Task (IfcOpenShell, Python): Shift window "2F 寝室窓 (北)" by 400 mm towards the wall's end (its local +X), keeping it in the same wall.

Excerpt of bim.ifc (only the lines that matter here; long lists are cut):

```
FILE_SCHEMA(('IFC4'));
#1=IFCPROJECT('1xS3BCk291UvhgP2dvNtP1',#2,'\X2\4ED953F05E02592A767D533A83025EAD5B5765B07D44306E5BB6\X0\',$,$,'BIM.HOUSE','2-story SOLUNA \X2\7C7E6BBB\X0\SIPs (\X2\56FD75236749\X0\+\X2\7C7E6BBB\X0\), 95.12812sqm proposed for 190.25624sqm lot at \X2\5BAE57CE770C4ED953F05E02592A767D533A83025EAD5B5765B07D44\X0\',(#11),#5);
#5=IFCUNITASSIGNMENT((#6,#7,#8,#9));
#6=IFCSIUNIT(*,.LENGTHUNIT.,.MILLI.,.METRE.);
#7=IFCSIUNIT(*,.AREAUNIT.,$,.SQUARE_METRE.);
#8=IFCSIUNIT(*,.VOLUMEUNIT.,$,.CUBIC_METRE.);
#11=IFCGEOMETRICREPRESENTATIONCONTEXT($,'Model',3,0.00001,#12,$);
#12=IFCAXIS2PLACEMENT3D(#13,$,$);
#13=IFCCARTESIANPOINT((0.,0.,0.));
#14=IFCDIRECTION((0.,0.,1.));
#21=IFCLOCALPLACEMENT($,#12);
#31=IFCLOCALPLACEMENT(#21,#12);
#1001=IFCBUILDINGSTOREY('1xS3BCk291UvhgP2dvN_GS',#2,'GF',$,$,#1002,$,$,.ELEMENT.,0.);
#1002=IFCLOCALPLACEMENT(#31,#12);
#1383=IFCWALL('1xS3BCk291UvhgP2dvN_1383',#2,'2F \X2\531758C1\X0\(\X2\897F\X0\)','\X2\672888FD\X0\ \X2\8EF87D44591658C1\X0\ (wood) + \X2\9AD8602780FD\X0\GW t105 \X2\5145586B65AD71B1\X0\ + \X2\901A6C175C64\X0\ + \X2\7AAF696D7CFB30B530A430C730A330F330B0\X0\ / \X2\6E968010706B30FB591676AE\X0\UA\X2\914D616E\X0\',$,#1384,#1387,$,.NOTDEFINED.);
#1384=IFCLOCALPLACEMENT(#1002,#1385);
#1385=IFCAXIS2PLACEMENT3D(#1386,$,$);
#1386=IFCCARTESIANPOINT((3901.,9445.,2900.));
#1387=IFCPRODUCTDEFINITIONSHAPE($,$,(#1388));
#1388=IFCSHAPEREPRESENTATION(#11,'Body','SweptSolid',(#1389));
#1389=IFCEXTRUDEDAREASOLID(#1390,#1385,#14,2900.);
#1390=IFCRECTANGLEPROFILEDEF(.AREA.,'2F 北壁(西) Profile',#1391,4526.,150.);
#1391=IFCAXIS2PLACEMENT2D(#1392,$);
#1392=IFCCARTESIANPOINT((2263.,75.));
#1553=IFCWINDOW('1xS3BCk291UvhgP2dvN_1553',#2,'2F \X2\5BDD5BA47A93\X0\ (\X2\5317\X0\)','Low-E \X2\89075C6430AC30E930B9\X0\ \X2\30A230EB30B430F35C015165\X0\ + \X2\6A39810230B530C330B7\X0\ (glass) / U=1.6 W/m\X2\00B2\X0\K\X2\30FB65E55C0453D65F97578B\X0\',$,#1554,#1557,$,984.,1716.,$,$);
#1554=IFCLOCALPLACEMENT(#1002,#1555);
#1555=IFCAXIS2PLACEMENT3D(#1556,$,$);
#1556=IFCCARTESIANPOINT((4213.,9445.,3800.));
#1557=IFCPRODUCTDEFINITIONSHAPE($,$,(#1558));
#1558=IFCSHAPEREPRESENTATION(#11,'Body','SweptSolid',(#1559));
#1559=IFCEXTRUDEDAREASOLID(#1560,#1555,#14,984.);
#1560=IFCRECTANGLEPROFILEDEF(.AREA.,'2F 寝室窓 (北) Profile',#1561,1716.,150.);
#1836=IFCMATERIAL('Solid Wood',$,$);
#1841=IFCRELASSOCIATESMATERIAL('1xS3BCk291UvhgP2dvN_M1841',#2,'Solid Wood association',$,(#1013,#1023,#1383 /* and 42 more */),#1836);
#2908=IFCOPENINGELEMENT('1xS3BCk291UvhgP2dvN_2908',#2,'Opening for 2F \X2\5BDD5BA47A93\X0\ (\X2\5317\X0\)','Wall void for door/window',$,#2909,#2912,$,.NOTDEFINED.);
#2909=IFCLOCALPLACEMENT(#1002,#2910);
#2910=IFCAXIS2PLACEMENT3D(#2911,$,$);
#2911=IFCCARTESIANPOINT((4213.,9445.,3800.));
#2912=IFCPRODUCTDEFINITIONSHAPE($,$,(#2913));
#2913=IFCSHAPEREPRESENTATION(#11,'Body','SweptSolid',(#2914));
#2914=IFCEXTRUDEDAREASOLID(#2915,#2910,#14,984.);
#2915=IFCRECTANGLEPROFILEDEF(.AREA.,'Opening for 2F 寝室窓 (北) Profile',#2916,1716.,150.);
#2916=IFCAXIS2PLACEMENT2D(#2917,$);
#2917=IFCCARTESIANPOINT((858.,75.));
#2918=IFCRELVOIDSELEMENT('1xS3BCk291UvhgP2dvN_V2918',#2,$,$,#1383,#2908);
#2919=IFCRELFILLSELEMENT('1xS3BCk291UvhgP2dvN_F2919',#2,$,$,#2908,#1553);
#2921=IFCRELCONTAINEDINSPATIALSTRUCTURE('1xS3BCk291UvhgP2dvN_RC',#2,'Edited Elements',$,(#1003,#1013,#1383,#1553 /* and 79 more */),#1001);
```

```python
import ifcopenshell
import ifcopenshell.api.geometry
import ifcopenshell.util.placement
import ifcopenshell.util.unit

model = ifcopenshell.open("bim.ifc")
unit_scale = ifcopenshell.util.unit.calculate_unit_scale(model)

window = model.by_id(1553)
opening = window.FillsVoids[0].RelatingOpeningElement
wall = opening.VoidsElements[0].RelatingBuildingElement

wall_matrix = ifcopenshell.util.placement.get_local_placement(wall.ObjectPlacement)
shift = wall_matrix[:3, 0] * 0.4 / unit_scale
before = ifcopenshell.util.placement.get_local_placement(window.ObjectPlacement)[:3, 3].copy()

# The window is not placed relative to its opening, so move both.
for product in (opening, window):
    matrix = ifcopenshell.util.placement.get_local_placement(product.ObjectPlacement)
    matrix[:3, 3] += shift
    ifcopenshell.api.geometry.edit_object_placement(model, product=product, matrix=matrix, is_si=False)

after = ifcopenshell.util.placement.get_local_placement(window.ObjectPlacement)[:3, 3]
print("window moved by", (after - before).round(3) + 0.0)

model.write("bim-out.ifc")
```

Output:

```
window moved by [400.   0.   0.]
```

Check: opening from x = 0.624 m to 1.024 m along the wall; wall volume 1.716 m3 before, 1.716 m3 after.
